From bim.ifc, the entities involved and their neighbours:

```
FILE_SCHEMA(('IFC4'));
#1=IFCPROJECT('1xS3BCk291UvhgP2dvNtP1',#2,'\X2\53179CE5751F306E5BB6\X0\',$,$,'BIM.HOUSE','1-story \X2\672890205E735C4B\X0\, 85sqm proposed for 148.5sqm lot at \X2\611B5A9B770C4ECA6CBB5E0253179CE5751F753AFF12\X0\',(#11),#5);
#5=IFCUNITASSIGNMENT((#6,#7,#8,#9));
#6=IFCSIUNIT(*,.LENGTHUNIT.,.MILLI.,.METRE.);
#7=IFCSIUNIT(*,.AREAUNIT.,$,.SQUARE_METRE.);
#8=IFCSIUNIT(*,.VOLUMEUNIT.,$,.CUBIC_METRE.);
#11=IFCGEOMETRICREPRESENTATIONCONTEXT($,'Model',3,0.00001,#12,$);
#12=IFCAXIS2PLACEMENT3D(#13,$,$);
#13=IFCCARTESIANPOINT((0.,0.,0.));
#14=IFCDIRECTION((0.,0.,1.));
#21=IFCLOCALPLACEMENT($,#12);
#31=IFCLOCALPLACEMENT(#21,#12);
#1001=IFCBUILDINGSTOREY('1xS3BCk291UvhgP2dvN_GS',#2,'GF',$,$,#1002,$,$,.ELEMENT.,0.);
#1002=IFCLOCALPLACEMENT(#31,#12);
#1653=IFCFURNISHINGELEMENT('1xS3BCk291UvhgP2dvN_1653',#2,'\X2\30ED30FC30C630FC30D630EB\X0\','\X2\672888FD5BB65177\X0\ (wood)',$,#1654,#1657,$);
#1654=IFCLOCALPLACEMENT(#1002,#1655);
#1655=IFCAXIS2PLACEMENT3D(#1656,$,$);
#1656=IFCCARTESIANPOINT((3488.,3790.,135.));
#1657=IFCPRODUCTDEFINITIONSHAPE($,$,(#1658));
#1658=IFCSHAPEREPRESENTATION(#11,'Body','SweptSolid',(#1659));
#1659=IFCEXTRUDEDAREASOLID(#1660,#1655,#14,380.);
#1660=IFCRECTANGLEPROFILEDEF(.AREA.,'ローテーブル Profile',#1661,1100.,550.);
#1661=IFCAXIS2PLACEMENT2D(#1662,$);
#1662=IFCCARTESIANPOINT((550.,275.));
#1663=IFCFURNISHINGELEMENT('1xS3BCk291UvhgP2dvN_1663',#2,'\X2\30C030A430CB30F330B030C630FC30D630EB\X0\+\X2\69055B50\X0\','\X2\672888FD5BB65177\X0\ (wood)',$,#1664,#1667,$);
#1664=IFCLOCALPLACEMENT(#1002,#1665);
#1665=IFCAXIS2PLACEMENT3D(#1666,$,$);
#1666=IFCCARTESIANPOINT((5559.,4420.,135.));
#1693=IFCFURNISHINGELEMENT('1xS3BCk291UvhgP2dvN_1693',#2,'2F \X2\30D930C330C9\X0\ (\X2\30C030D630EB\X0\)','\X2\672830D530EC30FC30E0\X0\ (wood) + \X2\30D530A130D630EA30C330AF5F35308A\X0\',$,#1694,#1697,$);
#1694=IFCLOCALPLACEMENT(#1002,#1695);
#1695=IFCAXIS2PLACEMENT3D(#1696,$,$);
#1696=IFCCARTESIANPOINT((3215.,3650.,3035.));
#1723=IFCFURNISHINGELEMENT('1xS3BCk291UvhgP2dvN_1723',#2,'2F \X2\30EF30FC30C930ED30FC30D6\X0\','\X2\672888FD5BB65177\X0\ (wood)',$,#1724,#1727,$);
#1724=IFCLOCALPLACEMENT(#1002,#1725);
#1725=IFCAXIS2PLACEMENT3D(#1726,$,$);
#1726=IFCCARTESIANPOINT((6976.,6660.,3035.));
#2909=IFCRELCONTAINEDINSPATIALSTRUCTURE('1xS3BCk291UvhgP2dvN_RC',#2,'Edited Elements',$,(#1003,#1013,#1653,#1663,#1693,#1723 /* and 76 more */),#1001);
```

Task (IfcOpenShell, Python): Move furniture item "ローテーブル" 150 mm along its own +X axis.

```python
import ifcopenshell
import ifcopenshell.api.geometry
import ifcopenshell.util.placement

model = ifcopenshell.open("bim.ifc")

item = model.by_guid("1xS3BCk291UvhgP2dvN_1653")
matrix = ifcopenshell.util.placement.get_local_placement(item.ObjectPlacement)
matrix[:3, 3] += matrix[:3, 0] * 150.0
ifcopenshell.api.geometry.edit_object_placement(model, product=item, matrix=matrix, is_si=False)

print(ifcopenshell.util.placement.get_local_placement(item.ObjectPlacement).round(3) + 0.0)

model.write("bim_v2.ifc")
```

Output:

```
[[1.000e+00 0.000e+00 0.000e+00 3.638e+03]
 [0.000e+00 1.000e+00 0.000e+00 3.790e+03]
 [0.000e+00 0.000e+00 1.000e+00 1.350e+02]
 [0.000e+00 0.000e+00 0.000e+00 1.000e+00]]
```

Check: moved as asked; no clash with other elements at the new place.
